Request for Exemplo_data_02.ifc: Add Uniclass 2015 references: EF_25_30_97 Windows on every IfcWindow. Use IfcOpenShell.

First a look at what the model holds.

```python
import ifcopenshell

model = ifcopenshell.open("Exemplo_data_02.ifc")
print(model.schema)
print("classifications:", [c.Name for c in model.by_type("IfcClassification")])
for ifc_class in ("IfcDoor", "IfcRoof", "IfcStair", "IfcWall", "IfcWindow"):
    print(ifc_class, len(model.by_type(ifc_class)))
```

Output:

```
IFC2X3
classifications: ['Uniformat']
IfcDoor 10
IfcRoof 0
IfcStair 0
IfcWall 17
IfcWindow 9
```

```python
import ifcopenshell
import ifcopenshell.api.classification

model = ifcopenshell.open("Exemplo_data_02.ifc")

# IFC2X3 requires Source and Edition and has no link from the project to the system.
system = model.create_entity("IfcClassification", Source="NBS", Edition="2015", Name="Uniclass 2015")

codes = {
    "IfcWindow": ("EF_25_30_97", "Windows"),
}
for ifc_class, (code, name) in codes.items():
    products = model.by_type(ifc_class)
    ifcopenshell.api.classification.add_reference(
        model, products=products, classification=system, identification=code, name=name
    )
    print(code, len(products))

model.write("Exemplo_data_02_rev.ifc")
```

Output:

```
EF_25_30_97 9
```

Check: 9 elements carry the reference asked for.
